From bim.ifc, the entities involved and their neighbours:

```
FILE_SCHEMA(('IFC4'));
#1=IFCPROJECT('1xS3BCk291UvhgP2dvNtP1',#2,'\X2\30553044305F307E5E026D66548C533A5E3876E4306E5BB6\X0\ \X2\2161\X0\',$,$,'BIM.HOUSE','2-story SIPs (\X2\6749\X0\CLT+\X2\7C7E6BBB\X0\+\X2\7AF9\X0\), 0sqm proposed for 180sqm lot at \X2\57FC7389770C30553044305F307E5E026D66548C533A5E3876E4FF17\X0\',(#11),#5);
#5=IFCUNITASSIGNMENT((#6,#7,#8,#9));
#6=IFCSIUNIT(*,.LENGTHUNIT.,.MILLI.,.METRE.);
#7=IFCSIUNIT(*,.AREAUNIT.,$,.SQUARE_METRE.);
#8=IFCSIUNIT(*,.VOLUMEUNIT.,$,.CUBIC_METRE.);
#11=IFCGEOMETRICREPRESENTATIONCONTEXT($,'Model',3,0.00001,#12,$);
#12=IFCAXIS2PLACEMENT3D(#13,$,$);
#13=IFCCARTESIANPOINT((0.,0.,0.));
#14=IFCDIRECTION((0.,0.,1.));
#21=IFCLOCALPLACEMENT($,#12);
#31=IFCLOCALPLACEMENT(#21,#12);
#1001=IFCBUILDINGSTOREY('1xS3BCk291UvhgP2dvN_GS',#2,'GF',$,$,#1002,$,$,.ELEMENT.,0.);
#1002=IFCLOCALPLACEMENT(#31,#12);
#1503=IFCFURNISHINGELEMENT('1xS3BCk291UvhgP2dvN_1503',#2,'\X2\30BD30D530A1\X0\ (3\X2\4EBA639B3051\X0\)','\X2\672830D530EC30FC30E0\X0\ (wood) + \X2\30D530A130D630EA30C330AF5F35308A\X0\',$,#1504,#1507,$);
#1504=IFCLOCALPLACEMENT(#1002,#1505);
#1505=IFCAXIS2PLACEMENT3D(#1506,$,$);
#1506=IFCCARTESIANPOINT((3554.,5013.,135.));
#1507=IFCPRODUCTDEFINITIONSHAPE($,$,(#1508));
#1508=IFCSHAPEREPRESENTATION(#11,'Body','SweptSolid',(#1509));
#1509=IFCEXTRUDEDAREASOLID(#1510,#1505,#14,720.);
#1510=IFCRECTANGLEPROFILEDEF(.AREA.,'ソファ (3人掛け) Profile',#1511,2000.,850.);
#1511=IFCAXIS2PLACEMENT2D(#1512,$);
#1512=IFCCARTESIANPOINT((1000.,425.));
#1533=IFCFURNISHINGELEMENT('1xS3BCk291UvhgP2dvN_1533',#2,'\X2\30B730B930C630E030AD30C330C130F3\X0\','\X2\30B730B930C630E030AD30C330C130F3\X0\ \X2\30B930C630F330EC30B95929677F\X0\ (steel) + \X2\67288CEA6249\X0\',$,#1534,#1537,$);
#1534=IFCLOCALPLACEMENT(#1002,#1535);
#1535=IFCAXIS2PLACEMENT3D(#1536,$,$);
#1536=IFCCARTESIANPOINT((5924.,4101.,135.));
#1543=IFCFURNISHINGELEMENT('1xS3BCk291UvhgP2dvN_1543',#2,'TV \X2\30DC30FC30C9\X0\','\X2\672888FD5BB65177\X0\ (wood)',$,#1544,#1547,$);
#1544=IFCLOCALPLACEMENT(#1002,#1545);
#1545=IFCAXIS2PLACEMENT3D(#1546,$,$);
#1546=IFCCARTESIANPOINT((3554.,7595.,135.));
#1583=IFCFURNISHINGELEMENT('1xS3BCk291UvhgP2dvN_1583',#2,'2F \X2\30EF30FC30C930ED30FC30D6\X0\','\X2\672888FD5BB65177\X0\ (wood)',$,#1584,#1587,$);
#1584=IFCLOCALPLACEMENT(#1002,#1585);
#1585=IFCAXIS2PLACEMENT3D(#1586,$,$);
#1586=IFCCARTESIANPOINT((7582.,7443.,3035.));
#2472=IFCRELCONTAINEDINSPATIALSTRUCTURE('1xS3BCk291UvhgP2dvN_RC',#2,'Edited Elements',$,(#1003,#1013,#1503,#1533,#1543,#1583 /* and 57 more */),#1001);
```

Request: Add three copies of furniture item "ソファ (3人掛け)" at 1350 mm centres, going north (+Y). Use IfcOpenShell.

```python
import numpy as np
import ifcopenshell
import ifcopenshell.api.geometry
import ifcopenshell.api.root
import ifcopenshell.util.element
import ifcopenshell.util.placement

model = ifcopenshell.open("bim.ifc")


def reuse_history(source, copy):
    """copy_class also copies each property set's owner history, people and application; keep the originals."""
    for rel in copy.IsDefinedBy:
        if rel.is_a("IfcRelDefinesByProperties") and (history := rel.RelatingPropertyDefinition.OwnerHistory):
            rel.RelatingPropertyDefinition.OwnerHistory = source.OwnerHistory
            ifcopenshell.util.element.remove_deep2(model, history)


source = model.by_guid("1xS3BCk291UvhgP2dvN_1503")
base = ifcopenshell.util.placement.get_local_placement(source.ObjectPlacement)
step = np.array([0.0, 1.0, 0.0]) * 1350.0

for i in range(1, 4):
    copy = ifcopenshell.api.root.copy_class(model, product=source)
    copy.Representation = ifcopenshell.util.element.copy_deep(
        model, source.Representation, exclude=["IfcGeometricRepresentationContext", "IfcRepresentationMap"]
    )
    reuse_history(source, copy)
    matrix = base.copy()
    matrix[:3, 3] += i * step
    print("added at", matrix[:3, 3].round(3) + 0.0)
    ifcopenshell.api.geometry.edit_object_placement(model, product=copy, matrix=matrix, is_si=False)

model.write("bim_v2.ifc")
```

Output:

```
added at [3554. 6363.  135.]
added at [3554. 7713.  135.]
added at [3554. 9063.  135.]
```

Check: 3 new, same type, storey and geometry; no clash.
